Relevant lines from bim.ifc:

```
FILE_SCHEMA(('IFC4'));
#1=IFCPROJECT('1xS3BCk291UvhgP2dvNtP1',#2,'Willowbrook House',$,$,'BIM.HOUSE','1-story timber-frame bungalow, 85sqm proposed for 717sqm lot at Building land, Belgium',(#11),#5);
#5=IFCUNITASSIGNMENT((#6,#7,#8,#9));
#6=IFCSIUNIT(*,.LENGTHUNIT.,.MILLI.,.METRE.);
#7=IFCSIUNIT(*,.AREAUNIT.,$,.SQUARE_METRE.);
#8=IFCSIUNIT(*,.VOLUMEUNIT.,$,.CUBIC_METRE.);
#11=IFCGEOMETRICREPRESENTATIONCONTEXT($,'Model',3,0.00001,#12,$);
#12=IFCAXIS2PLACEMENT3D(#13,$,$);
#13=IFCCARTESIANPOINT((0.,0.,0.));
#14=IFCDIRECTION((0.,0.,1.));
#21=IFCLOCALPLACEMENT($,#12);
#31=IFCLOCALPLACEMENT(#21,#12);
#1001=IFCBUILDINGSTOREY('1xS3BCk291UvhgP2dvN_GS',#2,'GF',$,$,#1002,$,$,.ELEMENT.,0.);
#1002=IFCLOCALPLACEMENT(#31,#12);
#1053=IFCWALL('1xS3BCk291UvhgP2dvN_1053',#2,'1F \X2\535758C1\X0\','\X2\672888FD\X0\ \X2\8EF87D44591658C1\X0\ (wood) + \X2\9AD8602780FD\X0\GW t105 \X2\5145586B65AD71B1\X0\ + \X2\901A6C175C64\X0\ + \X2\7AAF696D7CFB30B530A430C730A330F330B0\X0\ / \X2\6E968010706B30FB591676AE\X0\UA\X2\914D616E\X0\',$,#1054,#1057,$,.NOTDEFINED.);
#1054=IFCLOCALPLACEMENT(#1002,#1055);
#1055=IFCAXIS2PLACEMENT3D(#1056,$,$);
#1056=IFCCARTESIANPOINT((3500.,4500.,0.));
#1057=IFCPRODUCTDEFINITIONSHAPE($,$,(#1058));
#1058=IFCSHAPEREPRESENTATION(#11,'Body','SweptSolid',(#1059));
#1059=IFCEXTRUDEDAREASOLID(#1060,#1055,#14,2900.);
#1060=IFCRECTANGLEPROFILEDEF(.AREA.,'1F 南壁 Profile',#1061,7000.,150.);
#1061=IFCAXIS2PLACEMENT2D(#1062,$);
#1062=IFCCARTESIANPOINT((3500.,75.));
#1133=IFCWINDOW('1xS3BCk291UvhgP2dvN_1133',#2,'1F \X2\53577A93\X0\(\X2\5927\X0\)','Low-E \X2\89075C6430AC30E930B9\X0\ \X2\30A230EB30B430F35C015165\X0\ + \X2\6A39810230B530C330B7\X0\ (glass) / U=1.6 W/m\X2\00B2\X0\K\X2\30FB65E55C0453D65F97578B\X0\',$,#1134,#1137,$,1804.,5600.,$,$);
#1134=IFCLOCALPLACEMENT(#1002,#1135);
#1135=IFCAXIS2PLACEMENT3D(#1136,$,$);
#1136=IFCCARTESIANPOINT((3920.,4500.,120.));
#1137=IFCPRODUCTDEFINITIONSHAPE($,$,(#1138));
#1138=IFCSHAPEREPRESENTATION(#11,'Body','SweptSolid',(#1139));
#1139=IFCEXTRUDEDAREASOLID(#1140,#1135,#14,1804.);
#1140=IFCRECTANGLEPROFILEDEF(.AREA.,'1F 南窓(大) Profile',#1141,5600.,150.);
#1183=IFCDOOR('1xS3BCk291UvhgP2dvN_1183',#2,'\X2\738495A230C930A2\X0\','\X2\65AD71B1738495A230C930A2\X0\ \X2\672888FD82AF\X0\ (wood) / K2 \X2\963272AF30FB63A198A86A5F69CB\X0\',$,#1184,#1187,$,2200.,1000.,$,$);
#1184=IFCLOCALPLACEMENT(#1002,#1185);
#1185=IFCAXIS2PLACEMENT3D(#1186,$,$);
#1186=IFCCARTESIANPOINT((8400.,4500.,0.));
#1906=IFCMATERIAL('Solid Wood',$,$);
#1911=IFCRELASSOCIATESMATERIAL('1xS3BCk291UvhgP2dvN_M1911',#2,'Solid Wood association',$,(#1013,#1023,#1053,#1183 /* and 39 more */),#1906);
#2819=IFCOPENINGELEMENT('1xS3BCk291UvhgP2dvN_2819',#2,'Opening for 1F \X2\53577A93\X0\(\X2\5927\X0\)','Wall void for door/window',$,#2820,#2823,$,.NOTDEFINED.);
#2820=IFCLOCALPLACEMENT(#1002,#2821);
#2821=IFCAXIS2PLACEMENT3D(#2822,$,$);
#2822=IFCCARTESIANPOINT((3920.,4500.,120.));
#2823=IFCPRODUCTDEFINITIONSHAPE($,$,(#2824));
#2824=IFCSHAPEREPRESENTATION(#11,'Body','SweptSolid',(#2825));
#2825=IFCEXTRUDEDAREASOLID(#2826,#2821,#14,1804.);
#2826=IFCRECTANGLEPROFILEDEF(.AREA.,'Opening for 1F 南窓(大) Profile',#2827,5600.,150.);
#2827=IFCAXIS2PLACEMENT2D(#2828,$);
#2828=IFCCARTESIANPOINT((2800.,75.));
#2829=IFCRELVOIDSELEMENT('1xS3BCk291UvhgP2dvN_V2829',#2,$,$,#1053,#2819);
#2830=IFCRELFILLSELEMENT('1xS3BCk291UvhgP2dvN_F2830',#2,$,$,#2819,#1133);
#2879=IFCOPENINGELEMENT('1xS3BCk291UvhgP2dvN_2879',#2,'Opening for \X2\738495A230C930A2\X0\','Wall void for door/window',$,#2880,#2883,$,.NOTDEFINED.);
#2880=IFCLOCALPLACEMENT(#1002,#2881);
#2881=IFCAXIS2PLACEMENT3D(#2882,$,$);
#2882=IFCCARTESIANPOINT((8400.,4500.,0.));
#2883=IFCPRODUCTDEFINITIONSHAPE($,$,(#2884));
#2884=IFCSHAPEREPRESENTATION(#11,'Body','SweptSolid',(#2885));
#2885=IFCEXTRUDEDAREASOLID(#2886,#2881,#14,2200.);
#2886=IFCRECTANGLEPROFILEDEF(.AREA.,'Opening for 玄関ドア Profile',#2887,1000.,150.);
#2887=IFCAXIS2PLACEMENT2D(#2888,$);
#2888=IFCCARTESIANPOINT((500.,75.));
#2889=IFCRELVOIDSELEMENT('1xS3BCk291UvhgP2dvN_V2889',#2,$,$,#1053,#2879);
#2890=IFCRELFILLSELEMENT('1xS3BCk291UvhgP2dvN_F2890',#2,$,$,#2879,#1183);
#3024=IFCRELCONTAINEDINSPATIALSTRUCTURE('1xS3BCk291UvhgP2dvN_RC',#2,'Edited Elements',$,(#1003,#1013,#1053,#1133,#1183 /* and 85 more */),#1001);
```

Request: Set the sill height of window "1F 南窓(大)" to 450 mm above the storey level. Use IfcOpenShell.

```python
import numpy as np
import ifcopenshell
import ifcopenshell.api.geometry
import ifcopenshell.geom
import ifcopenshell.util.element
import ifcopenshell.util.placement
import ifcopenshell.util.shape
import ifcopenshell.util.unit

model = ifcopenshell.open("bim.ifc")
unit_scale = ifcopenshell.util.unit.calculate_unit_scale(model)

window = model.by_id(1133)
opening = window.FillsVoids[0].RelatingOpeningElement
storey = ifcopenshell.util.element.get_container(window, ifc_class="IfcBuildingStorey")
level = ifcopenshell.util.placement.get_local_placement(storey.ObjectPlacement)[2, 3]

# The opening's origin need not be at the sill, so measure its lowest point.
shape = ifcopenshell.geom.create_shape(ifcopenshell.geom.settings(), opening)
bottom = ifcopenshell.util.shape.get_shape_bottom_elevation(shape, shape.geometry) / unit_scale
dz = level + 450.0 - bottom

shift = np.array([0.0, 0.0, dz])
# The window is not placed relative to its opening, so move both.
for product in (opening, window):
    matrix = ifcopenshell.util.placement.get_local_placement(product.ObjectPlacement)
    matrix[:3, 3] += shift
    ifcopenshell.api.geometry.edit_object_placement(model, product=product, matrix=matrix, is_si=False)

print(f"moved by {dz * unit_scale:+.3f} m")

model.write("bim_updated.ifc")
```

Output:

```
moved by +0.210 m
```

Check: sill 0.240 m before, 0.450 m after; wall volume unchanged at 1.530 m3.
